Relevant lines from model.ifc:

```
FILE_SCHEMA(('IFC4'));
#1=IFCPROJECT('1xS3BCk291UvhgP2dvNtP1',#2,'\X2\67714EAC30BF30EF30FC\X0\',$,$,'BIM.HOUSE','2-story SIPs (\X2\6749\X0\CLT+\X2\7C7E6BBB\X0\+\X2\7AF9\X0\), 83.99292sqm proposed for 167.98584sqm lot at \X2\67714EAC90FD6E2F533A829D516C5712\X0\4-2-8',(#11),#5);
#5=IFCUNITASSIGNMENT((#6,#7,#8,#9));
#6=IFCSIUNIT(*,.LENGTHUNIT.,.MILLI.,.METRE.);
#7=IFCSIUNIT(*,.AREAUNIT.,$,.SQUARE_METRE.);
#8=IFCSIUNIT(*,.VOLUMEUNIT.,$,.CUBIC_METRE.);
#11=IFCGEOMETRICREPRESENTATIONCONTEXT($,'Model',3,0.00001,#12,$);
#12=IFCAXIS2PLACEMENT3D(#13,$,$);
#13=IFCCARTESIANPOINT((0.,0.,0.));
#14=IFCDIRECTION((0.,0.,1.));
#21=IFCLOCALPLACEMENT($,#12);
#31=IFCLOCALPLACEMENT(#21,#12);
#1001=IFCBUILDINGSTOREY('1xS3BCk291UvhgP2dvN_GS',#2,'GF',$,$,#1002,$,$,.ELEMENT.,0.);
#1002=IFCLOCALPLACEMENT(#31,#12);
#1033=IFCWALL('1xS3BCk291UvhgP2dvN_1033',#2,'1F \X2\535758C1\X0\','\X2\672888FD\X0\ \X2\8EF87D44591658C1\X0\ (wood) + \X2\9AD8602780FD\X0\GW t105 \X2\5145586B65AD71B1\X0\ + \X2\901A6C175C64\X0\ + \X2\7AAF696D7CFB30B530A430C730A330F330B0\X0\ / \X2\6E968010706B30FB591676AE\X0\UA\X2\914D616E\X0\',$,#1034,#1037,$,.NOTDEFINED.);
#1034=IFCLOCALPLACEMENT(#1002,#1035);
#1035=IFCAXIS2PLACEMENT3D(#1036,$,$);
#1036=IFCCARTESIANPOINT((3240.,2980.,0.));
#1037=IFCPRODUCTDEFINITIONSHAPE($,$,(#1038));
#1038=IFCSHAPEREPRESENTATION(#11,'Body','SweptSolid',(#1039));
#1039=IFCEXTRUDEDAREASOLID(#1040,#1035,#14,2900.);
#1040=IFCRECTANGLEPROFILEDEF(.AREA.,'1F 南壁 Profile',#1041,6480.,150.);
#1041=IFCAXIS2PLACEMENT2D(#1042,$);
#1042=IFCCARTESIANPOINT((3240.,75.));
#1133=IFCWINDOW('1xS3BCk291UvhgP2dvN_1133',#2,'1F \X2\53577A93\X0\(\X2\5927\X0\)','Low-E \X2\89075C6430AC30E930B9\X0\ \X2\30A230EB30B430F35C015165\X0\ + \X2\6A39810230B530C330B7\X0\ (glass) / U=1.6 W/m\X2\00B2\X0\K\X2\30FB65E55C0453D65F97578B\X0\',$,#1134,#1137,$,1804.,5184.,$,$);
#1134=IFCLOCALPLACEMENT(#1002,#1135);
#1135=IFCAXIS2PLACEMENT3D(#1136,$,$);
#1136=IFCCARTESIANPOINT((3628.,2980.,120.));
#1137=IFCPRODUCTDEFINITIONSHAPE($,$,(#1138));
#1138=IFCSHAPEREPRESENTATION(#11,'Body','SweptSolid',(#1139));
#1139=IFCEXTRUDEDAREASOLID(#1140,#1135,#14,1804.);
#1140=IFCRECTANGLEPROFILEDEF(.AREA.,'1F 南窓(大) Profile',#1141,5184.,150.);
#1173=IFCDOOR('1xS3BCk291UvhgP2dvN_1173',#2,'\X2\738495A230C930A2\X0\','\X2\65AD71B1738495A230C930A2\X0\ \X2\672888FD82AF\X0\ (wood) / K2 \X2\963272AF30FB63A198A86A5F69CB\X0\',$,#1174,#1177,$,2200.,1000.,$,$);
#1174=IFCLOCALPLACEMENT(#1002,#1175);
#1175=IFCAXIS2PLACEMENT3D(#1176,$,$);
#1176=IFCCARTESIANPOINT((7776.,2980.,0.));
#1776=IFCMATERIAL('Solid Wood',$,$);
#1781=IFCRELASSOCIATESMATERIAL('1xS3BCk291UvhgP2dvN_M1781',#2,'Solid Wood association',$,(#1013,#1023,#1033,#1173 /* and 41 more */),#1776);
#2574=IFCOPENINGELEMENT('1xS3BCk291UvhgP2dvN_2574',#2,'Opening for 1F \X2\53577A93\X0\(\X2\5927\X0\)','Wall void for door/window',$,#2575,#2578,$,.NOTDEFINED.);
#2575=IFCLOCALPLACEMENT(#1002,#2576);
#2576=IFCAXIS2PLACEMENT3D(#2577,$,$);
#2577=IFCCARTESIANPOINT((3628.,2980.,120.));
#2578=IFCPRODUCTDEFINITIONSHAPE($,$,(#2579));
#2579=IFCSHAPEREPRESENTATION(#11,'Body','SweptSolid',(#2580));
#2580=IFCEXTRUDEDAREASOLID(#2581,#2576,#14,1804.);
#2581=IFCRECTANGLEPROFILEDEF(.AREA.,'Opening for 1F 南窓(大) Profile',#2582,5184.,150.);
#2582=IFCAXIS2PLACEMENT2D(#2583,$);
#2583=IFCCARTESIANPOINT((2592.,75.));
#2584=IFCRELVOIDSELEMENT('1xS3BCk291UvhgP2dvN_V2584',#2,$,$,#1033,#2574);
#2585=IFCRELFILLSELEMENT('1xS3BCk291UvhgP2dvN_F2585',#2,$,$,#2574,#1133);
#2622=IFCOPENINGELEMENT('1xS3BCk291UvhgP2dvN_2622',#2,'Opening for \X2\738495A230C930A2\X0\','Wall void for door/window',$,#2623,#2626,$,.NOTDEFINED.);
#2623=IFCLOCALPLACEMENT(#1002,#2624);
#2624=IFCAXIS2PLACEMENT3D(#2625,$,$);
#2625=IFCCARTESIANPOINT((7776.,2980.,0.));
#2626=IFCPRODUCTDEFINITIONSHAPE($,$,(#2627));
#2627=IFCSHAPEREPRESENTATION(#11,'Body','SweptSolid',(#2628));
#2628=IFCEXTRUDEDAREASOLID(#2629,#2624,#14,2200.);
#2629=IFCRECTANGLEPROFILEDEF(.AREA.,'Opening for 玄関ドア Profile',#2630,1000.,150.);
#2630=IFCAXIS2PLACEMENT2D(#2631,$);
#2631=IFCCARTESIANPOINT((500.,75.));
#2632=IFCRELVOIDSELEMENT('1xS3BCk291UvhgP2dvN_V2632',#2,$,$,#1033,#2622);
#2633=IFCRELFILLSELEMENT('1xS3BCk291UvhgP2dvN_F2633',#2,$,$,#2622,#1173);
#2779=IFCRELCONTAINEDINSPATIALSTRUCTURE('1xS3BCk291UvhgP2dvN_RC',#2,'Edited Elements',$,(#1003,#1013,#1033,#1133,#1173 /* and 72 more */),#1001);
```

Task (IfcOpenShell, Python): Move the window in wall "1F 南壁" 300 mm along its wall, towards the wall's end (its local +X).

```python
import ifcopenshell
import ifcopenshell.api.geometry
import ifcopenshell.util.placement

model = ifcopenshell.open("model.ifc")

window = model.by_guid("1xS3BCk291UvhgP2dvN_1133")
opening = window.FillsVoids[0].RelatingOpeningElement
wall = opening.VoidsElements[0].RelatingBuildingElement

wall_matrix = ifcopenshell.util.placement.get_local_placement(wall.ObjectPlacement)
shift = wall_matrix[:3, 0] * 300.0
before = ifcopenshell.util.placement.get_local_placement(window.ObjectPlacement)[:3, 3].copy()

# The window is not placed relative to its opening, so move both.
for product in (opening, window):
    matrix = ifcopenshell.util.placement.get_local_placement(product.ObjectPlacement)
    matrix[:3, 3] += shift
    ifcopenshell.api.geometry.edit_object_placement(model, product=product, matrix=matrix, is_si=False)

after = ifcopenshell.util.placement.get_local_placement(window.ObjectPlacement)[:3, 3]
print("window moved by", (after - before).round(3) + 0.0)

model.write("model-out.ifc")
```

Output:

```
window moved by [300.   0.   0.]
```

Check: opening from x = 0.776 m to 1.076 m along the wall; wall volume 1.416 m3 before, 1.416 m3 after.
